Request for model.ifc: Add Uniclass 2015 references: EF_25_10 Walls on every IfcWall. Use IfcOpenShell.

First a look at what the model holds.

```python
import ifcopenshell

model = ifcopenshell.open("model.ifc")
print(model.schema)
print("classifications:", [c.Name for c in model.by_type("IfcClassification")])
for ifc_class in ("IfcDoor", "IfcRoof", "IfcStair", "IfcWall", "IfcWindow"):
    print(ifc_class, len(model.by_type(ifc_class)))
```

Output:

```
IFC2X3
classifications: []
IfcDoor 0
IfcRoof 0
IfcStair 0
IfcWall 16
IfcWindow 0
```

```python
import ifcopenshell
import ifcopenshell.api.classification

model = ifcopenshell.open("model.ifc")

# IFC2X3 requires Source and Edition and has no link from the project to the system.
system = model.create_entity("IfcClassification", Source="NBS", Edition="2015", Name="Uniclass 2015")

codes = {
    "IfcWall": ("EF_25_10", "Walls"),
}
for ifc_class, (code, name) in codes.items():
    products = model.by_type(ifc_class)
    ifcopenshell.api.classification.add_reference(
        model, products=products, classification=system, identification=code, name=name
    )
    print(code, len(products))

model.write("model_edited.ifc")
```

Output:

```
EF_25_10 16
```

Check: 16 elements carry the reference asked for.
